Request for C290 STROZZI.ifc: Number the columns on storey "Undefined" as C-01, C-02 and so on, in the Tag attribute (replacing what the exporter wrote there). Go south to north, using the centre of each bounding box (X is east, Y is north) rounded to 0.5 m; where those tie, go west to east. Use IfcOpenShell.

First a look at what the model holds.

```python
import ifcopenshell
import ifcopenshell.util.element
import ifcopenshell.util.placement

model = ifcopenshell.open("C290 STROZZI.ifc")
print(model.schema)
storey = next(s for s in model.by_type("IfcBuildingStorey") if s.Name == "Undefined")
columns = [e for e in ifcopenshell.util.element.get_decomposition(storey) if e.is_a("IfcColumn")]
for e in sorted(columns, key=lambda e: e.id()):
    origin = ifcopenshell.util.placement.get_local_placement(e.ObjectPlacement)[:3, 3]
    print(e.id(), e.Tag, e.Name, origin.round(2) + 0.0, sep=" | ")
```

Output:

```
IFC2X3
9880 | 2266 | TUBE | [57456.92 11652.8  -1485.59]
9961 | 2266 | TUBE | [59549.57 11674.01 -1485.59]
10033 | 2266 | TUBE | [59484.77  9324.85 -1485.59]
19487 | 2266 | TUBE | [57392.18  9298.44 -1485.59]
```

```python
import ifcopenshell
import ifcopenshell.geom
import ifcopenshell.util.element
import ifcopenshell.util.shape

model = ifcopenshell.open("C290 STROZZI.ifc")
settings = ifcopenshell.geom.settings()
settings.set("use-world-coords", True)


def centre(element):
    shape = ifcopenshell.geom.create_shape(settings, element)
    return ifcopenshell.util.shape.get_bbox_centroid(shape.geometry)


storey = next(s for s in model.by_type("IfcBuildingStorey") if s.Name == "Undefined")
columns = [e for e in ifcopenshell.util.element.get_decomposition(storey) if e.is_a("IfcColumn")]

# Insertion points can sit at a corner or the storey origin, so sort by the geometry (in metres).
centres = {e: centre(e) for e in columns}
columns.sort(key=lambda e: (round(centres[e][1] / 0.5), centres[e][0]))

for i, e in enumerate(columns, start=1):
    number = f"C-{i:02d}"
    e.Tag = number
    print(e.id(), number)

model.write("C290 STROZZI_rev.ifc")
```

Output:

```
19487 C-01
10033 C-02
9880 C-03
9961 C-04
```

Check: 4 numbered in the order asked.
